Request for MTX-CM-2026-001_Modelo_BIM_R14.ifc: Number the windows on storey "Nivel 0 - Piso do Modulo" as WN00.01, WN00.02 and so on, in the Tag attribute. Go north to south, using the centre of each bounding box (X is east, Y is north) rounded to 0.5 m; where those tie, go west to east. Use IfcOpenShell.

First a look at what the model holds.

```python
import ifcopenshell
import ifcopenshell.util.element
import ifcopenshell.util.placement

model = ifcopenshell.open("MTX-CM-2026-001_Modelo_BIM_R14.ifc")
print(model.schema)
storey = next(s for s in model.by_type("IfcBuildingStorey") if s.Name == "Nivel 0 - Piso do Modulo")
windows = [e for e in ifcopenshell.util.element.get_decomposition(storey) if e.is_a("IfcWindow")]
for e in sorted(windows, key=lambda e: e.id()):
    origin = ifcopenshell.util.placement.get_local_placement(e.ObjectPlacement)[:3, 3]
    print(e.id(), e.Tag, e.Name, origin.round(2) + 0.0, sep=" | ")
```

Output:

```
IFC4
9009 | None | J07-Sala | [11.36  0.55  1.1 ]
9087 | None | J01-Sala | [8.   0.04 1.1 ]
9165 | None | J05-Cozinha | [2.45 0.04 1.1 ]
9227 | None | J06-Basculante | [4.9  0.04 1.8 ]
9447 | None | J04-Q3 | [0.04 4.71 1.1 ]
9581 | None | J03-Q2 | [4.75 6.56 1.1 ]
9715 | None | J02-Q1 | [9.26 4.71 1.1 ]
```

```python
import ifcopenshell
import ifcopenshell.geom
import ifcopenshell.util.element
import ifcopenshell.util.shape

model = ifcopenshell.open("MTX-CM-2026-001_Modelo_BIM_R14.ifc")
settings = ifcopenshell.geom.settings()
settings.set("use-world-coords", True)


def centre(element):
    shape = ifcopenshell.geom.create_shape(settings, element)
    return ifcopenshell.util.shape.get_bbox_centroid(shape.geometry)


storey = next(s for s in model.by_type("IfcBuildingStorey") if s.Name == "Nivel 0 - Piso do Modulo")
windows = [e for e in ifcopenshell.util.element.get_decomposition(storey) if e.is_a("IfcWindow")]

# Insertion points can sit at a corner or the storey origin, so sort by the geometry (in metres).
centres = {e: centre(e) for e in windows}
windows.sort(key=lambda e: (-round(centres[e][1] / 0.5), centres[e][0]))

for i, e in enumerate(windows, start=1):
    number = f"WN00.{i:02d}"
    e.Tag = number
    print(e.id(), number)

model.write("MTX-CM-2026-001_Modelo_BIM_R14_edited.ifc")
```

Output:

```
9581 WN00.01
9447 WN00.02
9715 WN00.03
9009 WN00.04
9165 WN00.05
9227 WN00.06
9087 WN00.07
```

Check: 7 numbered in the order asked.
